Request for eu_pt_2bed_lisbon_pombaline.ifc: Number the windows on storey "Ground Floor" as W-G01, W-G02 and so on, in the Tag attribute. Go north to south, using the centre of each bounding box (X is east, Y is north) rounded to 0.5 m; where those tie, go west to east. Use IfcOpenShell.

First a look at what the model holds.

```python
import ifcopenshell
import ifcopenshell.util.element
import ifcopenshell.util.placement

model = ifcopenshell.open("eu_pt_2bed_lisbon_pombaline.ifc")
print(model.schema)
storey = next(s for s in model.by_type("IfcBuildingStorey") if s.Name == "Ground Floor")
windows = [e for e in ifcopenshell.util.element.get_decomposition(storey) if e.is_a("IfcWindow")]
for e in sorted(windows, key=lambda e: e.id()):
    origin = ifcopenshell.util.placement.get_local_placement(e.ObjectPlacement)[:3, 3]
    print(e.id(), e.Tag, e.Name, origin.round(2) + 0.0, sep=" | ")
```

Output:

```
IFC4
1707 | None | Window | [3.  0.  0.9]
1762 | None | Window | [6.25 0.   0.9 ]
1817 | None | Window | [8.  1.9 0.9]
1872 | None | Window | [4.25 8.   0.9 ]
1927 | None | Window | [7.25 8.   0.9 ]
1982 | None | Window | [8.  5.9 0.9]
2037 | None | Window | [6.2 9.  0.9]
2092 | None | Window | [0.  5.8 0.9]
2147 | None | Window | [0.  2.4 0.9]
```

```python
import ifcopenshell
import ifcopenshell.geom
import ifcopenshell.util.element
import ifcopenshell.util.shape

model = ifcopenshell.open("eu_pt_2bed_lisbon_pombaline.ifc")
settings = ifcopenshell.geom.settings()
settings.set("use-world-coords", True)


def centre(element):
    shape = ifcopenshell.geom.create_shape(settings, element)
    return ifcopenshell.util.shape.get_bbox_centroid(shape.geometry)


storey = next(s for s in model.by_type("IfcBuildingStorey") if s.Name == "Ground Floor")
windows = [e for e in ifcopenshell.util.element.get_decomposition(storey) if e.is_a("IfcWindow")]

# Insertion points can sit at a corner or the storey origin, so sort by the geometry (in metres).
centres = {e: centre(e) for e in windows}
windows.sort(key=lambda e: (-round(centres[e][1] / 0.5), centres[e][0]))

for i, e in enumerate(windows, start=1):
    number = f"W-G{i:02d}"
    e.Tag = number
    print(e.id(), number)

model.write("eu_pt_2bed_lisbon_pombaline_updated.ifc")
```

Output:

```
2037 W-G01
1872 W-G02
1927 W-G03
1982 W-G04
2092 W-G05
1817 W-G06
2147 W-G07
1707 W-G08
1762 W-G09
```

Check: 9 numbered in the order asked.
